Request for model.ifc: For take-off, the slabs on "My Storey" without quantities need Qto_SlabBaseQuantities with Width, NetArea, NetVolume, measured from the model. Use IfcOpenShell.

First a look at what the model holds.

```python
import ifcopenshell
import ifcopenshell.util.element
import ifcopenshell.util.unit

model = ifcopenshell.open("model.ifc")
print(model.schema)
for unit_type in ("LENGTHUNIT", "AREAUNIT", "VOLUMEUNIT"):
    print(unit_type, ifcopenshell.util.unit.calculate_unit_scale(model, unit_type))
storey = next(s for s in model.by_type("IfcBuildingStorey") if s.Name == "My Storey")
slabs = [e for e in ifcopenshell.util.element.get_decomposition(storey) if e.is_a("IfcSlab")]
for e in sorted(slabs, key=lambda e: e.id()):
    print(e.id(), e.is_a(), e.Name, list(ifcopenshell.util.element.get_psets(e, qtos_only=True)), sep=" | ")
```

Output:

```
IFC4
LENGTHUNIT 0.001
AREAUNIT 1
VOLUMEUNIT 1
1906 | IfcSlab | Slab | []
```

```python
import ifcopenshell
import ifcopenshell.api.pset
import ifcopenshell.geom
import ifcopenshell.util.element
import ifcopenshell.util.shape
import ifcopenshell.util.unit

model = ifcopenshell.open("model.ifc")
unit_scale = ifcopenshell.util.unit.calculate_unit_scale(model)
area_scale = ifcopenshell.util.unit.calculate_unit_scale(model, "AREAUNIT")
volume_scale = ifcopenshell.util.unit.calculate_unit_scale(model, "VOLUMEUNIT")
settings = ifcopenshell.geom.settings()

storey = next(s for s in model.by_type("IfcBuildingStorey") if s.Name == "My Storey")
slabs = [e for e in ifcopenshell.util.element.get_decomposition(storey) if e.is_a("IfcSlab")]

for e in sorted(slabs, key=lambda e: e.id()):
    if ifcopenshell.util.element.get_psets(e, qtos_only=True, should_inherit=False):
        continue
    # Geometry comes back in metres, in the element's own axes.
    shape = ifcopenshell.geom.create_shape(settings, e)
    values = {
        "Width": ifcopenshell.util.shape.get_z(shape.geometry) / unit_scale,
        "NetArea": ifcopenshell.util.shape.get_footprint_area(shape.geometry) / area_scale,
        "NetVolume": ifcopenshell.util.shape.get_volume(shape.geometry) / volume_scale,
    }
    qto = ifcopenshell.api.pset.add_qto(model, product=e, name="Qto_SlabBaseQuantities")
    ifcopenshell.api.pset.edit_qto(model, qto=qto, properties=values)
    print(e.id(), {k: round(v, 3) for k, v in values.items()})

model.write("model_edited.ifc")
```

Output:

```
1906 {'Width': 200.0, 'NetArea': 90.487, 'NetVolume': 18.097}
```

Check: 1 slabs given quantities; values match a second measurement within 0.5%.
